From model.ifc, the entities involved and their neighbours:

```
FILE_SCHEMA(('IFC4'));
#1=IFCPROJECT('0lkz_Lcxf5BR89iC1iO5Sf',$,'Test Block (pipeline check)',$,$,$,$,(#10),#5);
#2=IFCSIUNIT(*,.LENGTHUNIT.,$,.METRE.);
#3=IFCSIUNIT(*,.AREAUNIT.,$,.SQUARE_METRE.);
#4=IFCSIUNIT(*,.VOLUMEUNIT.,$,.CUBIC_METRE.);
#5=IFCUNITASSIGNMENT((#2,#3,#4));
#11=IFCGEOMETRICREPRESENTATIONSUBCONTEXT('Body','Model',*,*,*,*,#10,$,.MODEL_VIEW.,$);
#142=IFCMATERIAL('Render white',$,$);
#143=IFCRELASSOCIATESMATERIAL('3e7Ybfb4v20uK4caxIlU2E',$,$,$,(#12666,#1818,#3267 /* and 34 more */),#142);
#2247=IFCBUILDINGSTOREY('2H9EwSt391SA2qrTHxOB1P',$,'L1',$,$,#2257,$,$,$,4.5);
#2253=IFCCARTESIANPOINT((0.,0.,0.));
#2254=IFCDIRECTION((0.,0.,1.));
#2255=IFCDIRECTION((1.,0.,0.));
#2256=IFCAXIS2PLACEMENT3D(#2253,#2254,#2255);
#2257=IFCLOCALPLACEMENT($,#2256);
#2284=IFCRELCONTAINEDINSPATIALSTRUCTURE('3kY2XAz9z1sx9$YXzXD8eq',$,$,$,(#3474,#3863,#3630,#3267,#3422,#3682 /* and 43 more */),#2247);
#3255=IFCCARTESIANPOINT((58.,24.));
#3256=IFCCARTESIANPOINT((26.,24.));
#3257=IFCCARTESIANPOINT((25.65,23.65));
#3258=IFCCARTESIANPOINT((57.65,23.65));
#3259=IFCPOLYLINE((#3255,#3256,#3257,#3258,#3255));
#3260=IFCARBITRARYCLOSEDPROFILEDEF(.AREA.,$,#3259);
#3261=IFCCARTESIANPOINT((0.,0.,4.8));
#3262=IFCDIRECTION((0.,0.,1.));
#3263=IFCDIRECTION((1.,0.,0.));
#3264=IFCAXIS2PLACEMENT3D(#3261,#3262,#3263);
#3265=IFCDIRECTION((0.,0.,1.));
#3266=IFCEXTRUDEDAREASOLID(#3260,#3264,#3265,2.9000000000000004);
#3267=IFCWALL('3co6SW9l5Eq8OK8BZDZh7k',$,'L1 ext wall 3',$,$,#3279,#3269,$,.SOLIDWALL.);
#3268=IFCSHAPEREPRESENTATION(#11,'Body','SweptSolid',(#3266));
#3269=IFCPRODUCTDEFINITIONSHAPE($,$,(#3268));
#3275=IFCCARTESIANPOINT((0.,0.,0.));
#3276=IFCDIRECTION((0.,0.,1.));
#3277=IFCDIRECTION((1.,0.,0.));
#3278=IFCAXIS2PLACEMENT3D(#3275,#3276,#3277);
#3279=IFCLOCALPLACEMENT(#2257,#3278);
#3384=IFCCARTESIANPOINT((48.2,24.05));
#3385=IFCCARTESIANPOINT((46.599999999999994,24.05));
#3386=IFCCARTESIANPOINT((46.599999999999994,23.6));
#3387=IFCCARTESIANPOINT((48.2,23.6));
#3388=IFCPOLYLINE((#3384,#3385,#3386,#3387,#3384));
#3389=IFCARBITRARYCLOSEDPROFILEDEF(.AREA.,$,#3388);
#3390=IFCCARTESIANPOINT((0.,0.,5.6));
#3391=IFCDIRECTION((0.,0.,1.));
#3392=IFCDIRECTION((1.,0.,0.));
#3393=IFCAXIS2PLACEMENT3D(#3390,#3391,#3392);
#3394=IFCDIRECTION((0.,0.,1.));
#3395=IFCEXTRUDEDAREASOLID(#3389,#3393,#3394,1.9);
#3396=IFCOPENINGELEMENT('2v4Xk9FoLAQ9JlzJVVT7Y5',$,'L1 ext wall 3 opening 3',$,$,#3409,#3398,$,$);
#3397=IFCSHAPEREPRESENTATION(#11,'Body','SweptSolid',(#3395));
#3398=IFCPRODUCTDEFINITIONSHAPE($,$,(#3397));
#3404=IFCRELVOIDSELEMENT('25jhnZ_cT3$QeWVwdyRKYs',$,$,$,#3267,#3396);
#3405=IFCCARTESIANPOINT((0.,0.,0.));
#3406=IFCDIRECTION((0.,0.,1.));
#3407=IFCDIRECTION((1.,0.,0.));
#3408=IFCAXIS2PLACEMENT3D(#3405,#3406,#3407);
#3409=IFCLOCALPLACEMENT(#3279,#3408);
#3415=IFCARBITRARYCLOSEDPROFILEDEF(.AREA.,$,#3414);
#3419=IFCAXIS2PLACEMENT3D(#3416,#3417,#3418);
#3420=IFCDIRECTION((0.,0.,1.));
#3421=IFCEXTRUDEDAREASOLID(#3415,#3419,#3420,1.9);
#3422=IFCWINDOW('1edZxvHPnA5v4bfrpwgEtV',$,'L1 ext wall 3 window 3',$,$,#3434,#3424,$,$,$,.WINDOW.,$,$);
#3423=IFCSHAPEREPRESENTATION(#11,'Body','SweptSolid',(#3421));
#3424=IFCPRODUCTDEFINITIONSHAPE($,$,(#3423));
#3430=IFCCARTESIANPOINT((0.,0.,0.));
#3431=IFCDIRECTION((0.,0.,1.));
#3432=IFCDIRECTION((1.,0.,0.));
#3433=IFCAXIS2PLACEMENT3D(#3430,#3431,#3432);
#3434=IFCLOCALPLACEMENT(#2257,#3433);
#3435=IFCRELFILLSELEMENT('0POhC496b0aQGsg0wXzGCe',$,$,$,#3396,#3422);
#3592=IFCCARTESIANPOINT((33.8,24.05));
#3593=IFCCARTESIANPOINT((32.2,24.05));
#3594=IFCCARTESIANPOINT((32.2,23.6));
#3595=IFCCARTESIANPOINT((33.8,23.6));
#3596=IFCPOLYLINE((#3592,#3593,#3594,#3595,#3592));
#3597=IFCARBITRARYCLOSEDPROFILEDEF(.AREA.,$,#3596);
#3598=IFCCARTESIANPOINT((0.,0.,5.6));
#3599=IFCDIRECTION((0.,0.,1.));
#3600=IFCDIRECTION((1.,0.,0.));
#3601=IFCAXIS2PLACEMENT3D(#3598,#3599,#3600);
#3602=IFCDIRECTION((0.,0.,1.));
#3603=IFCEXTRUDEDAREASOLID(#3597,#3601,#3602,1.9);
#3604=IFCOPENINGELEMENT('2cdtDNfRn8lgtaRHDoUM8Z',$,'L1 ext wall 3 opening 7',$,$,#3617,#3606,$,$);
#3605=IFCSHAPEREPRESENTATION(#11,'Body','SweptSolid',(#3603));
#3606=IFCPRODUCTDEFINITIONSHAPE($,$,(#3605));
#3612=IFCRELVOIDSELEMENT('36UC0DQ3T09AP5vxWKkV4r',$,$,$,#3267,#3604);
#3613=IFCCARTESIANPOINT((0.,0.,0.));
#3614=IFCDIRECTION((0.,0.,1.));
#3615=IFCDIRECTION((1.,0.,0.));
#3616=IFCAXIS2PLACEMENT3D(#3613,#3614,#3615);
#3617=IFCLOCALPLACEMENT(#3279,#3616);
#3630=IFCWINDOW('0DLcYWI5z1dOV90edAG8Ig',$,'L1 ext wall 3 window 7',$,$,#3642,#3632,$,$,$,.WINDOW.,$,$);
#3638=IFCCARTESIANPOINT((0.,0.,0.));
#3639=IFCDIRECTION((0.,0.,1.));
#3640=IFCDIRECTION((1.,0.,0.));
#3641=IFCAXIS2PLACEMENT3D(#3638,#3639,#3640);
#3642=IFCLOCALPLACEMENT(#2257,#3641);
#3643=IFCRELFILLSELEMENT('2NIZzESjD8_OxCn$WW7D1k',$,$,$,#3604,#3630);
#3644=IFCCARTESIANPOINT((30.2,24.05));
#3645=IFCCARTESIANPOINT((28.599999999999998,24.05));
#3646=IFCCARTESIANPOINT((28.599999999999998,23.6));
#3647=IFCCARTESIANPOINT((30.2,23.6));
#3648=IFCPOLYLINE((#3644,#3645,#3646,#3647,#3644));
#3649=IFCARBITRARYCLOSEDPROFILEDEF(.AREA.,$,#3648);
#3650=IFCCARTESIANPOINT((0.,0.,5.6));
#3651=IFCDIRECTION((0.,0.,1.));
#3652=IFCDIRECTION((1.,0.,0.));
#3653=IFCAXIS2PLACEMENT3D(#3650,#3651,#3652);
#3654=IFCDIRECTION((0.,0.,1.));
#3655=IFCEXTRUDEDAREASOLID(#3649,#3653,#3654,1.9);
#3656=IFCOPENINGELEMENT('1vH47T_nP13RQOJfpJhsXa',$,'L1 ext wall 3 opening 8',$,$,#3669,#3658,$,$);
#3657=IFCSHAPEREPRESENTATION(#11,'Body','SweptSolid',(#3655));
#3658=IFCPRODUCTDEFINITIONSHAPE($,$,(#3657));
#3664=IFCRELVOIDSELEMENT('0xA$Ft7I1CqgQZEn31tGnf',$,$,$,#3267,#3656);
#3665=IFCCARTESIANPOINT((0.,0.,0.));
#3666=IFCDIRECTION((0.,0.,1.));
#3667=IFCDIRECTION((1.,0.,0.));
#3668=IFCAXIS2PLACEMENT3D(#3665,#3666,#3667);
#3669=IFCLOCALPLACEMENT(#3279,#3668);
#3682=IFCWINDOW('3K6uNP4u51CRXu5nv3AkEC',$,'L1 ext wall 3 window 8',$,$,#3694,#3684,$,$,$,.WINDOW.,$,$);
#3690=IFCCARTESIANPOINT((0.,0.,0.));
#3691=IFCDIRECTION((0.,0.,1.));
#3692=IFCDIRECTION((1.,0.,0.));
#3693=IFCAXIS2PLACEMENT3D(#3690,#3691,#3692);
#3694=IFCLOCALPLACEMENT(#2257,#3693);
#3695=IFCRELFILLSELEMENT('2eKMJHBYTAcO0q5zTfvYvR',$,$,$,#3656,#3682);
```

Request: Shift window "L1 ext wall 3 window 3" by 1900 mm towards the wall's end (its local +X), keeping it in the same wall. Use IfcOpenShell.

```python
import ifcopenshell
import ifcopenshell.api.geometry
import ifcopenshell.util.placement
import ifcopenshell.util.unit

model = ifcopenshell.open("model.ifc")
unit_scale = ifcopenshell.util.unit.calculate_unit_scale(model)

window = model.by_id(3422)
opening = window.FillsVoids[0].RelatingOpeningElement
wall = opening.VoidsElements[0].RelatingBuildingElement

wall_matrix = ifcopenshell.util.placement.get_local_placement(wall.ObjectPlacement)
shift = wall_matrix[:3, 0] * 1.9 / unit_scale
before = ifcopenshell.util.placement.get_local_placement(window.ObjectPlacement)[:3, 3].copy()

# The window is not placed relative to its opening, so move both.
for product in (opening, window):
    matrix = ifcopenshell.util.placement.get_local_placement(product.ObjectPlacement)
    matrix[:3, 3] += shift
    ifcopenshell.api.geometry.edit_object_placement(model, product=product, matrix=matrix, is_si=False)

after = ifcopenshell.util.placement.get_local_placement(window.ObjectPlacement)[:3, 3]
print("window moved by", (after - before).round(3) + 0.0)

model.write("model_rev.ifc")
```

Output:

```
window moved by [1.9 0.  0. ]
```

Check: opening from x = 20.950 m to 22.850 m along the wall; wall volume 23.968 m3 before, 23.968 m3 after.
